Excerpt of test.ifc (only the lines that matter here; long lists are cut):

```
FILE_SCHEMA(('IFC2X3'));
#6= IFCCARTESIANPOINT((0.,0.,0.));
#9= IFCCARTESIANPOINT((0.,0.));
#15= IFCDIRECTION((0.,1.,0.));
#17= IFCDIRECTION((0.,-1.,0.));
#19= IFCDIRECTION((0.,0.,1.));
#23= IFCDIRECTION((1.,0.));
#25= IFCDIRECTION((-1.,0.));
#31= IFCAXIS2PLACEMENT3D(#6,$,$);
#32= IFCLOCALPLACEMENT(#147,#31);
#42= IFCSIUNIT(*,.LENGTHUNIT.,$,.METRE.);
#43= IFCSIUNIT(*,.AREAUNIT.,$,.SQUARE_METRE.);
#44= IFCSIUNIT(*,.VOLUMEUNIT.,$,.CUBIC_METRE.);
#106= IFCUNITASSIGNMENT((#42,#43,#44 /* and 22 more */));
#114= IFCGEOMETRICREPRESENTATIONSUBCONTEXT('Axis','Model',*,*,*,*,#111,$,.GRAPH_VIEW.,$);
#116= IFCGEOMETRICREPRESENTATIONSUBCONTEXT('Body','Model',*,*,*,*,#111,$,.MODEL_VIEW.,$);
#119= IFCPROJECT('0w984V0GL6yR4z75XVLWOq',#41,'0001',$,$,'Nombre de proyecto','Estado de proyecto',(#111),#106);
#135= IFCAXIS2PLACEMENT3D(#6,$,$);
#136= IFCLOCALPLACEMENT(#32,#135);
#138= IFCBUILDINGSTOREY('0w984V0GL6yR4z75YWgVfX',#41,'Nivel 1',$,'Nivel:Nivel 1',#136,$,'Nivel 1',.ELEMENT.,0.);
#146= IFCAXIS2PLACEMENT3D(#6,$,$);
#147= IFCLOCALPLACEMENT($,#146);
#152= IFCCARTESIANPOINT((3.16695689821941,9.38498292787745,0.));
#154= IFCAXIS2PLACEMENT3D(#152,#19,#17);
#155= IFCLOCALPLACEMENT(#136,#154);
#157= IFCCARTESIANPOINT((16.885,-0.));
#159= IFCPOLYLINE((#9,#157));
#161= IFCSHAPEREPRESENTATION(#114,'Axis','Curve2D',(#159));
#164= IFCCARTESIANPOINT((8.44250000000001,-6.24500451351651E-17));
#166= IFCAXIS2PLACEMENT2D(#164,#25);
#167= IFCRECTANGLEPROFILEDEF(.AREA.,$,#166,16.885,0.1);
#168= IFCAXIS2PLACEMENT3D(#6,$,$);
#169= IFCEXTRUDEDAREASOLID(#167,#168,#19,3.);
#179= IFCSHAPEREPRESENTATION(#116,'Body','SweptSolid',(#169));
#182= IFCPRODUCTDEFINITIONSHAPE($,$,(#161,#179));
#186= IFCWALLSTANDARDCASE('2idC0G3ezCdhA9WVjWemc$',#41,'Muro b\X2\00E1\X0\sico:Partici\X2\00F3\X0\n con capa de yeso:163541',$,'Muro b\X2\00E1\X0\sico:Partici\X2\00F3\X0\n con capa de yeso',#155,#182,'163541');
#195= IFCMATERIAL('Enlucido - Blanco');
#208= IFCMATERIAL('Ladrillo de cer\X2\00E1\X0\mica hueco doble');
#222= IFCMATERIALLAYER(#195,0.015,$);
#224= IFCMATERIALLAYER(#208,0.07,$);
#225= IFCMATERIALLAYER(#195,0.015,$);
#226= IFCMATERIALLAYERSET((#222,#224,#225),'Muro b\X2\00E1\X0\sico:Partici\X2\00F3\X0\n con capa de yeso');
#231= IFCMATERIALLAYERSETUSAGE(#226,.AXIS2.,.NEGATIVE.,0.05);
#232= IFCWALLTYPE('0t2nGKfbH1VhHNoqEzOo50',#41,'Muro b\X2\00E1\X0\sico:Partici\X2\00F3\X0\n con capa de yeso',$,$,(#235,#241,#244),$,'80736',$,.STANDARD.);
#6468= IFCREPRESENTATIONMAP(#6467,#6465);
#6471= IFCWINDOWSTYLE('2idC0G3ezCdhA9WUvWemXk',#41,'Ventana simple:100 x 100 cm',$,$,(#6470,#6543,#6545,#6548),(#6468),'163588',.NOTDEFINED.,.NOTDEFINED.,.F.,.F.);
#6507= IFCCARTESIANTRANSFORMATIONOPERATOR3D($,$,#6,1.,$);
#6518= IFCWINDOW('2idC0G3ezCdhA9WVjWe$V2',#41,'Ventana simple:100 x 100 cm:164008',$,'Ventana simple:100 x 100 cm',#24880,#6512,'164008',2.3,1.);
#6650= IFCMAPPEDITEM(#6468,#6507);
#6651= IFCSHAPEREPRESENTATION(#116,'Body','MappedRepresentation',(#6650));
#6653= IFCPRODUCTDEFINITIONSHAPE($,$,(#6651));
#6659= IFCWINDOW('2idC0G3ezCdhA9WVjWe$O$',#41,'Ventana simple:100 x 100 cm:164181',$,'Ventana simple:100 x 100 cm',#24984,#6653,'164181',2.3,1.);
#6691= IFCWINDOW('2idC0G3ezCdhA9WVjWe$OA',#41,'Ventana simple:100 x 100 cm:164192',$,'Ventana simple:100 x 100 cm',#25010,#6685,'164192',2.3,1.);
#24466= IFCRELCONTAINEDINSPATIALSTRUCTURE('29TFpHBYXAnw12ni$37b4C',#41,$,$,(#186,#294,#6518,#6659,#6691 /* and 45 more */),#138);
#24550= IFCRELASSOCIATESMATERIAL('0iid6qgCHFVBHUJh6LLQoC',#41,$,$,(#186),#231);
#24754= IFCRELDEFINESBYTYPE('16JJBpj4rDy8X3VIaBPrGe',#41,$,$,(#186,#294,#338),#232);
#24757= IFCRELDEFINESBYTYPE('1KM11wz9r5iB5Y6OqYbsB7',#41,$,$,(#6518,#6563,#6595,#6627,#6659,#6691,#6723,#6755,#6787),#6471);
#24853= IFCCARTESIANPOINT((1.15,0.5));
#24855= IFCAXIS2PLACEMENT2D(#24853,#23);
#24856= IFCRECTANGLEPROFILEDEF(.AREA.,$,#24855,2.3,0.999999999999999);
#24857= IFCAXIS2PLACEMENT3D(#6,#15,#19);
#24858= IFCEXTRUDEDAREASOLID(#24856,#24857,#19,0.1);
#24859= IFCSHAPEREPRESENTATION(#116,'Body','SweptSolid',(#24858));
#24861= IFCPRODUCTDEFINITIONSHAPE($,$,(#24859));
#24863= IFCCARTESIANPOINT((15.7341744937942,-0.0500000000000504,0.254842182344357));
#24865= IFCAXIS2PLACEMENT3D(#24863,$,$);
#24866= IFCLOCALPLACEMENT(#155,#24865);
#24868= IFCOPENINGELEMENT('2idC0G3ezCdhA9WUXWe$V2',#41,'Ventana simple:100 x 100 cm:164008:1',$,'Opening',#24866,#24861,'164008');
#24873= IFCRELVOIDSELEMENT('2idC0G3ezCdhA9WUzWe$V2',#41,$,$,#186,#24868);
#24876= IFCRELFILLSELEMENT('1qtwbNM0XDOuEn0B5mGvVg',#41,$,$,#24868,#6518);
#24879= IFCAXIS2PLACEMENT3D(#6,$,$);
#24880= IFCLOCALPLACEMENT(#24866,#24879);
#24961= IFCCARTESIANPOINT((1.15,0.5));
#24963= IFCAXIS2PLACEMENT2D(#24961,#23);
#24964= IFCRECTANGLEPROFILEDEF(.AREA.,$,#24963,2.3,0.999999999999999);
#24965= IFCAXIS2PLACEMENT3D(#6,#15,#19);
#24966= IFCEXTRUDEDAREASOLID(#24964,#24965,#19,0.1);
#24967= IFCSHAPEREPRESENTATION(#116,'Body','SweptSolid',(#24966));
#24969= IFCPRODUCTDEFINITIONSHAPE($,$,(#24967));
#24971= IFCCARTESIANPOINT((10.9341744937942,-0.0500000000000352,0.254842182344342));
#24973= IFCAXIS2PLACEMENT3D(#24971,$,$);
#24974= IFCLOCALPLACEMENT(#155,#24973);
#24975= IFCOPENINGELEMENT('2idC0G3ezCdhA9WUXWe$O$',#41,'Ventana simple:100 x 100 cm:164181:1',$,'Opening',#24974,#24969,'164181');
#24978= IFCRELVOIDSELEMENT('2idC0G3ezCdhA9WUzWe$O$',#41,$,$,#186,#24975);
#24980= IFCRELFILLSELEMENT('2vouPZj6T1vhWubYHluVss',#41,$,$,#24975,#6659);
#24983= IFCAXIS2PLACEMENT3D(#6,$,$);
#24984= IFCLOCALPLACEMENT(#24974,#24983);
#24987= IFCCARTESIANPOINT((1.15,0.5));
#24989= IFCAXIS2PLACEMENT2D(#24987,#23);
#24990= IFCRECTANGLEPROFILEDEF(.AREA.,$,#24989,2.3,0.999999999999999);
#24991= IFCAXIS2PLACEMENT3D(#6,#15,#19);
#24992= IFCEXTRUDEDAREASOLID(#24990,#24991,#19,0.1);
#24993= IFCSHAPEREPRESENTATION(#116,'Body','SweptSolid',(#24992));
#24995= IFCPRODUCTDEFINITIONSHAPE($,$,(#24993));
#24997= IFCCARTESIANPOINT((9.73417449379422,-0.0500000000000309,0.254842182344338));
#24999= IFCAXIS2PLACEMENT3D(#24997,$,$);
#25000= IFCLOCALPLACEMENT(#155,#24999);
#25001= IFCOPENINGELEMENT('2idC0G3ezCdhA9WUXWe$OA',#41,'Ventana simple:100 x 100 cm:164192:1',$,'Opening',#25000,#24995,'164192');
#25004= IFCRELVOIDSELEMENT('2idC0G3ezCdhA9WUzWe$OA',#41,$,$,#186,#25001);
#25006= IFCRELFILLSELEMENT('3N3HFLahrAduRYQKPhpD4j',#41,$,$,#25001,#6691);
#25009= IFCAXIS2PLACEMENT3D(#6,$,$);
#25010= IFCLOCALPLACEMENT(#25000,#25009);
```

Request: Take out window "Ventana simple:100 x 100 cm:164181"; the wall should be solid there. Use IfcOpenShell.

```python
import ifcopenshell
import ifcopenshell.api.feature
import ifcopenshell.api.root
import ifcopenshell.geom
import ifcopenshell.util.shape

model = ifcopenshell.open("test.ifc")
settings = ifcopenshell.geom.settings()


def volume(element):
    """Net volume in cubic metres, openings subtracted."""
    shape = ifcopenshell.geom.create_shape(settings, element)
    return ifcopenshell.util.shape.get_volume(shape.geometry)


window = model.by_guid("2idC0G3ezCdhA9WVjWe$O$")
opening = window.FillsVoids[0].RelatingOpeningElement
wall = opening.VoidsElements[0].RelatingBuildingElement
before = volume(wall)

ifcopenshell.api.root.remove_product(model, product=window)
ifcopenshell.api.feature.remove_feature(model, feature=opening)

after = volume(wall)

print(f"wall volume {before:.3f} -> {after:.3f} m3")

model.write("test-out.ifc")
```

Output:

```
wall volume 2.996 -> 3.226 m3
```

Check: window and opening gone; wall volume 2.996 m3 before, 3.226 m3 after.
